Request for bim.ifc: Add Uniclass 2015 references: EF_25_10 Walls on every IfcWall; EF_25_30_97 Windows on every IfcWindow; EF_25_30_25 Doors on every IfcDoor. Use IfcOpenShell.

First a look at what the model holds.

```python
import ifcopenshell

model = ifcopenshell.open("bim.ifc")
print(model.schema)
print("classifications:", [c.Name for c in model.by_type("IfcClassification")])
for ifc_class in ("IfcDoor", "IfcRoof", "IfcStair", "IfcWall", "IfcWindow"):
    print(ifc_class, len(model.by_type(ifc_class)))
```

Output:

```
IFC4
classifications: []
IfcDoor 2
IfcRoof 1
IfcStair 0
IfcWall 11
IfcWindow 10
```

```python
import ifcopenshell
import ifcopenshell.api.classification

model = ifcopenshell.open("bim.ifc")

system = ifcopenshell.api.classification.add_classification(model, classification="Uniclass 2015")

codes = {
    "IfcWall": ("EF_25_10", "Walls"),
    "IfcWindow": ("EF_25_30_97", "Windows"),
    "IfcDoor": ("EF_25_30_25", "Doors"),
}
for ifc_class, (code, name) in codes.items():
    products = model.by_type(ifc_class)
    ifcopenshell.api.classification.add_reference(
        model, products=products, classification=system, identification=code, name=name
    )
    print(code, len(products))

model.write("bim-out.ifc")
```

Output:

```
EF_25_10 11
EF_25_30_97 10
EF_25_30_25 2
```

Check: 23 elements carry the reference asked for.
